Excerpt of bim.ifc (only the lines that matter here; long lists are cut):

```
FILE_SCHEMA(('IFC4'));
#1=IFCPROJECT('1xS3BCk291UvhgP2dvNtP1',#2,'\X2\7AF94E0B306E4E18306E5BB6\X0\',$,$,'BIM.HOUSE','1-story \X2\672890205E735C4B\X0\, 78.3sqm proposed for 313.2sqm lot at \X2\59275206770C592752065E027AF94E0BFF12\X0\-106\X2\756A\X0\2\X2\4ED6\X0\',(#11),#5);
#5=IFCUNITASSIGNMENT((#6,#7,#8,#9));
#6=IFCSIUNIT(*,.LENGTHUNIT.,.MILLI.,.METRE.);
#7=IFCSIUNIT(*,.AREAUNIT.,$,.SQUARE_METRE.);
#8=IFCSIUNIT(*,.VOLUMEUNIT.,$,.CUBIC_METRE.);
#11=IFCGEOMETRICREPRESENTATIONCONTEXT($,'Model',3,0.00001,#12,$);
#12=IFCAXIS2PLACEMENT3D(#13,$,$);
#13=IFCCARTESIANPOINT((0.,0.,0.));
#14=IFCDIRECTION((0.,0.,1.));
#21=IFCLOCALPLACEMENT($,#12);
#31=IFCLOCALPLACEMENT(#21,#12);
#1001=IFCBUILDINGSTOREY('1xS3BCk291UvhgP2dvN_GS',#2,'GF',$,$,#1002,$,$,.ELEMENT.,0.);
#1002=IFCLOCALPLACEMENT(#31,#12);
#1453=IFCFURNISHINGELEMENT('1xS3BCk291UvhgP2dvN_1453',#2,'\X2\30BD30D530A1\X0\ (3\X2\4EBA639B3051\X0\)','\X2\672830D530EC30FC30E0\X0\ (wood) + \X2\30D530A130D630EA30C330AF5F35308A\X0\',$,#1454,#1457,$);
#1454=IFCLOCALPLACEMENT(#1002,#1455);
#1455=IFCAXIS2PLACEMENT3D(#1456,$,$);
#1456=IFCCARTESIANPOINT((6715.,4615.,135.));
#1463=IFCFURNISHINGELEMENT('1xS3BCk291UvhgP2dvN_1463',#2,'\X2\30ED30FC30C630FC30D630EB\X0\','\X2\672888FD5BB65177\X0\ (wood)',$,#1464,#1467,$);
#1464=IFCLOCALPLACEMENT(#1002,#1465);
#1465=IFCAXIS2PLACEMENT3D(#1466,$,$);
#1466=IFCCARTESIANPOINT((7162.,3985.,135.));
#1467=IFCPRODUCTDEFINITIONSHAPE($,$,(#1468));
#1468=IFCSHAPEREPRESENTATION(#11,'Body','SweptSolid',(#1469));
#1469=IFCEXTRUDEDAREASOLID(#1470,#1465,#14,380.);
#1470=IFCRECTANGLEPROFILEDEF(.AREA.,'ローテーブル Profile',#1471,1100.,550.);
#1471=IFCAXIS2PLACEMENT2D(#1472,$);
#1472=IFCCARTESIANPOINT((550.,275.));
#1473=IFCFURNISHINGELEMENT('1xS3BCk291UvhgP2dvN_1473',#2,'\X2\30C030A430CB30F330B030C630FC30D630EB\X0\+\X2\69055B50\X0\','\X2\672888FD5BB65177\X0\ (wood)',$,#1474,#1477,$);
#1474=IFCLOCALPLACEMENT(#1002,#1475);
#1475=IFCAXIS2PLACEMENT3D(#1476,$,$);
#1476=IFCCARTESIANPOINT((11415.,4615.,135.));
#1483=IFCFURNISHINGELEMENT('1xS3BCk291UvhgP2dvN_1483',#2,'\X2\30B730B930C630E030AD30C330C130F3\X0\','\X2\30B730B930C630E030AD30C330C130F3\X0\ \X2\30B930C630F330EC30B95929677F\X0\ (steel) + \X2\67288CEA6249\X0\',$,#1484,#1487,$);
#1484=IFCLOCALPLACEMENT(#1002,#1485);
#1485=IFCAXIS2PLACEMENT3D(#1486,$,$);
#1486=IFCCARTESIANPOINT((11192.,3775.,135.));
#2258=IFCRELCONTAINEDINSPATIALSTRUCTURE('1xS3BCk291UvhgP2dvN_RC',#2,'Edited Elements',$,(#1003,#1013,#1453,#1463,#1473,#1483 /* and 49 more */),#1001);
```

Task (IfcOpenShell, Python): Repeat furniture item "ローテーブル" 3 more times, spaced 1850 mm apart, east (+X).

```python
import numpy as np
import ifcopenshell
import ifcopenshell.api.geometry
import ifcopenshell.api.root
import ifcopenshell.util.element
import ifcopenshell.util.placement
import ifcopenshell.util.unit

model = ifcopenshell.open("bim.ifc")
unit_scale = ifcopenshell.util.unit.calculate_unit_scale(model)


def reuse_history(source, copy):
    """copy_class also copies each property set's owner history, people and application; keep the originals."""
    for rel in copy.IsDefinedBy:
        if rel.is_a("IfcRelDefinesByProperties") and (history := rel.RelatingPropertyDefinition.OwnerHistory):
            rel.RelatingPropertyDefinition.OwnerHistory = source.OwnerHistory
            ifcopenshell.util.element.remove_deep2(model, history)


source = model.by_guid("1xS3BCk291UvhgP2dvN_1463")
base = ifcopenshell.util.placement.get_local_placement(source.ObjectPlacement)
step = np.array([1.0, 0.0, 0.0]) * 1.85 / unit_scale

for i in range(1, 4):
    copy = ifcopenshell.api.root.copy_class(model, product=source)
    copy.Representation = ifcopenshell.util.element.copy_deep(
        model, source.Representation, exclude=["IfcGeometricRepresentationContext", "IfcRepresentationMap"]
    )
    reuse_history(source, copy)
    matrix = base.copy()
    matrix[:3, 3] += i * step
    print("added at", matrix[:3, 3].round(3) + 0.0)
    ifcopenshell.api.geometry.edit_object_placement(model, product=copy, matrix=matrix, is_si=False)

model.write("bim_rev.ifc")
```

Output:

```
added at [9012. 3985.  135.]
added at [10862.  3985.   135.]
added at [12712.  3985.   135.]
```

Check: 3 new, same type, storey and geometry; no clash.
